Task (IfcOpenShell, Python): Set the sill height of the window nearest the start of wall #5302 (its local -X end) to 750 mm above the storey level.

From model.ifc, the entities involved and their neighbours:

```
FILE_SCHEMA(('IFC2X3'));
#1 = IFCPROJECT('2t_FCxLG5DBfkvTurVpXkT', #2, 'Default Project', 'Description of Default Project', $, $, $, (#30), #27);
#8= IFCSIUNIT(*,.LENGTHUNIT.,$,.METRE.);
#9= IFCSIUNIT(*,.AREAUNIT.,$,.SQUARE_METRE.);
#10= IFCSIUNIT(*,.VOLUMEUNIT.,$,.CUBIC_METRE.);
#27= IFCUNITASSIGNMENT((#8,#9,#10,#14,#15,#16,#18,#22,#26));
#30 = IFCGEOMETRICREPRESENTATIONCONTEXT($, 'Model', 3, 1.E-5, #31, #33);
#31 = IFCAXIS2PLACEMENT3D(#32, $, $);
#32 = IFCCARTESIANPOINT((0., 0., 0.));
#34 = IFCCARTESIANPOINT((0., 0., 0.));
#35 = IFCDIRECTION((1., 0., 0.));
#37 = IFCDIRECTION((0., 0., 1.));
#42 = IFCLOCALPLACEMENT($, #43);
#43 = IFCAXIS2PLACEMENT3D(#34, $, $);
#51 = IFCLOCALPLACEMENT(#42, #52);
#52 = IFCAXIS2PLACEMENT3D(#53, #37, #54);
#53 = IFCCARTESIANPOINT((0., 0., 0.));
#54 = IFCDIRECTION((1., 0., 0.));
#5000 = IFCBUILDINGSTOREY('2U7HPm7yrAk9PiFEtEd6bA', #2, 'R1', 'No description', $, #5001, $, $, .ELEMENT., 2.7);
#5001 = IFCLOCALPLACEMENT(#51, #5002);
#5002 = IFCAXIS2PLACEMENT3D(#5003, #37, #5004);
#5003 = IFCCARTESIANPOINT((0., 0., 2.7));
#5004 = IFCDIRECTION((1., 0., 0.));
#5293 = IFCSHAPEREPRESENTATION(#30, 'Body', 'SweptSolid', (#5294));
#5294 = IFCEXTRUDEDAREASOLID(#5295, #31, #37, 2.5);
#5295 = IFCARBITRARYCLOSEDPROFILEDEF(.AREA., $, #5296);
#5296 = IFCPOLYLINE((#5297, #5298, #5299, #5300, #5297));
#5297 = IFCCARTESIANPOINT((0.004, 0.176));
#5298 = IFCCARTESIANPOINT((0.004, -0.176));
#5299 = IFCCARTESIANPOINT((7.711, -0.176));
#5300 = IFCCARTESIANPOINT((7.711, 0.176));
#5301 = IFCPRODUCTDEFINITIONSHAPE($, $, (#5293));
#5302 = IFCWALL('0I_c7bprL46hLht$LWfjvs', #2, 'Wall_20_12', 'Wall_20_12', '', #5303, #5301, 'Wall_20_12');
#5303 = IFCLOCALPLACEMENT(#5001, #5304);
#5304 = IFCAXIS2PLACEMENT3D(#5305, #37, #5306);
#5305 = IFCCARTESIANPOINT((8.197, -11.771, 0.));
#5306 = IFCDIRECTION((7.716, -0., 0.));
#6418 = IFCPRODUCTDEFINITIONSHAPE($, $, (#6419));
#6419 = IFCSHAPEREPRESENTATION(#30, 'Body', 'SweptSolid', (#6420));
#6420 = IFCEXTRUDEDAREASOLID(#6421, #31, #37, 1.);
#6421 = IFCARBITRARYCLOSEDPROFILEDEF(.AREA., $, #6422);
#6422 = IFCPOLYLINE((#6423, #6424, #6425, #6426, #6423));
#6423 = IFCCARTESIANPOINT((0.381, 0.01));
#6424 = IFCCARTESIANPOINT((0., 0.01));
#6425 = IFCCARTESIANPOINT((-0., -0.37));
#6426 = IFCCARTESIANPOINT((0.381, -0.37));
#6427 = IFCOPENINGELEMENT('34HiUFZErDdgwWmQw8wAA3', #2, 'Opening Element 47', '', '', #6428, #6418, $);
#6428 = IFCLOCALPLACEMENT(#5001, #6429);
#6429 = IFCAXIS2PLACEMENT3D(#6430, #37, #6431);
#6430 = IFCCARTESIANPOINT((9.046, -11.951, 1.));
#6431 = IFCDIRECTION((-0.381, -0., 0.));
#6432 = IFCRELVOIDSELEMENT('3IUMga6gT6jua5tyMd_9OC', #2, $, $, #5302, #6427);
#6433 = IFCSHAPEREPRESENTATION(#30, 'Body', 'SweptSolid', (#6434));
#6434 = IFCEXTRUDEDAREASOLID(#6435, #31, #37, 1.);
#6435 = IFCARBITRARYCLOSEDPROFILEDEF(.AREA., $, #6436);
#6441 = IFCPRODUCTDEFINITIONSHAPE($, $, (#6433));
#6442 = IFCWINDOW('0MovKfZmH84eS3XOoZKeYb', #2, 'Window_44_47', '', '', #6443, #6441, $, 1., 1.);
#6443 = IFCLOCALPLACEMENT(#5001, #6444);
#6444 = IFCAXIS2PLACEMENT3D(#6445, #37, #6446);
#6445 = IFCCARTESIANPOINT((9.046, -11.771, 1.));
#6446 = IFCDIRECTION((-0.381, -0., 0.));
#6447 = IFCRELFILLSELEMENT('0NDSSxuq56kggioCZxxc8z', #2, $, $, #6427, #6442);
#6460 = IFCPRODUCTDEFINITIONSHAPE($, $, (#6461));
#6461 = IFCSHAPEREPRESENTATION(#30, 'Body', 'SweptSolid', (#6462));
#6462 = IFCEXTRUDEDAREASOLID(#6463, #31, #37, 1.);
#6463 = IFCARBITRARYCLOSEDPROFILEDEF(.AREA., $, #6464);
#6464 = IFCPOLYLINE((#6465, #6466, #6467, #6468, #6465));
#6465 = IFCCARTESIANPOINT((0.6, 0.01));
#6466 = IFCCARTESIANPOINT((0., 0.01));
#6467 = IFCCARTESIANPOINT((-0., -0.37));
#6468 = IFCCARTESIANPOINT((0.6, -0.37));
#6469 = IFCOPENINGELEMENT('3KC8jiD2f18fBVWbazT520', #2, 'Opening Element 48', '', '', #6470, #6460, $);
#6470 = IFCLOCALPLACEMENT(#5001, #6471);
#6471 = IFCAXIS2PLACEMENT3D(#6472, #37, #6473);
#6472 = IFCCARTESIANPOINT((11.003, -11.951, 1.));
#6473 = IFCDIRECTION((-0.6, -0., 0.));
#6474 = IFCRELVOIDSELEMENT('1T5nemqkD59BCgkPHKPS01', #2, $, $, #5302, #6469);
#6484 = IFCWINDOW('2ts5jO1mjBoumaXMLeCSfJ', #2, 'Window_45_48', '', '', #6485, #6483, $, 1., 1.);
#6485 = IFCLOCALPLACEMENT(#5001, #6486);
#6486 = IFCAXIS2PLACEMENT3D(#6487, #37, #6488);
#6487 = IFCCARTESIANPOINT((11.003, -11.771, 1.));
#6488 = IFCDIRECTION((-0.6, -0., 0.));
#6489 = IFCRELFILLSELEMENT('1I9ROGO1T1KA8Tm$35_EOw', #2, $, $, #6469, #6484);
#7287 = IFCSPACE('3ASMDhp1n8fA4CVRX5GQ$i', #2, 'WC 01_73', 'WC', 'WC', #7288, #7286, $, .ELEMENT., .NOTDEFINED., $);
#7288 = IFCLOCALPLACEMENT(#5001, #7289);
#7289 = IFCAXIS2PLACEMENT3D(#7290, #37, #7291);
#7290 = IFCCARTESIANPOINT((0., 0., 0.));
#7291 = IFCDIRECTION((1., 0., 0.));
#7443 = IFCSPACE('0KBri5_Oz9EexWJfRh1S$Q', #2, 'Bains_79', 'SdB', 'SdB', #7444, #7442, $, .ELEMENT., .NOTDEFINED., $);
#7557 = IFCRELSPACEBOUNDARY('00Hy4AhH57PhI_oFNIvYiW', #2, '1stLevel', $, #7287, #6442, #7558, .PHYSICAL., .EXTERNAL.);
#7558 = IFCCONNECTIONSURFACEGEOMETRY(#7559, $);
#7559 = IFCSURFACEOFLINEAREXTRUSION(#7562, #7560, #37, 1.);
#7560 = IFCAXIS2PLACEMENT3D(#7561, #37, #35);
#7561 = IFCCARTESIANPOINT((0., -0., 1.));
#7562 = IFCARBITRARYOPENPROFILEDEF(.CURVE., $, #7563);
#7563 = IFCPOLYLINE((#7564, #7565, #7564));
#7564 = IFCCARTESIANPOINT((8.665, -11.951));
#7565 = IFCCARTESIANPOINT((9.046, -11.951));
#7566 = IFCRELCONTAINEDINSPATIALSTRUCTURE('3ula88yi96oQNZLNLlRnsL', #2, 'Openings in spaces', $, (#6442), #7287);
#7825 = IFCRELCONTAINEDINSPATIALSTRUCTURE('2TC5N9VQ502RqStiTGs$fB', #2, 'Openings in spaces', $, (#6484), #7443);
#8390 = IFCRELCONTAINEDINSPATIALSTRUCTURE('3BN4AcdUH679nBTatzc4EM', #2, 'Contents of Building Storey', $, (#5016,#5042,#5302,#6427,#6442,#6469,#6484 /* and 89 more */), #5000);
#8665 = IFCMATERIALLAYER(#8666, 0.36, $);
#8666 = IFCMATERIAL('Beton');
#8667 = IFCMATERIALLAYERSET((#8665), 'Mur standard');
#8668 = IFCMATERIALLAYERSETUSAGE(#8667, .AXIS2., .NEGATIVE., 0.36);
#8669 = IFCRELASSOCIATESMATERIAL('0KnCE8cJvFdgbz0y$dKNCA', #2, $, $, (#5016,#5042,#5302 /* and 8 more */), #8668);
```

```python
import numpy as np
import ifcopenshell
import ifcopenshell.api.geometry
import ifcopenshell.geom
import ifcopenshell.util.element
import ifcopenshell.util.placement
import ifcopenshell.util.shape
import ifcopenshell.util.unit

model = ifcopenshell.open("model.ifc")
unit_scale = ifcopenshell.util.unit.calculate_unit_scale(model)

window = model.by_guid("0MovKfZmH84eS3XOoZKeYb")
opening = window.FillsVoids[0].RelatingOpeningElement
storey = ifcopenshell.util.element.get_container(window, ifc_class="IfcBuildingStorey")
level = ifcopenshell.util.placement.get_local_placement(storey.ObjectPlacement)[2, 3]

# The opening's origin need not be at the sill, so measure its lowest point.
shape = ifcopenshell.geom.create_shape(ifcopenshell.geom.settings(), opening)
bottom = ifcopenshell.util.shape.get_shape_bottom_elevation(shape, shape.geometry) / unit_scale
dz = level + 0.75 / unit_scale - bottom

shift = np.array([0.0, 0.0, dz])
# The window is not placed relative to its opening, so move both.
for product in (opening, window):
    matrix = ifcopenshell.util.placement.get_local_placement(product.ObjectPlacement)
    matrix[:3, 3] += shift
    ifcopenshell.api.geometry.edit_object_placement(model, product=product, matrix=matrix, is_si=False)

# Space boundary surfaces are stored in each space's coordinates; move them too.
for rel in window.ProvidesBoundaries:
    if not rel.ConnectionGeometry:
        continue
    surface = rel.ConnectionGeometry.SurfaceOnRelatingElement
    space_matrix = ifcopenshell.util.placement.get_local_placement(rel.RelatingSpace.ObjectPlacement)
    point = np.array(surface.Position.Location.Coordinates) + space_matrix[:3, :3].T @ shift
    surface.Position = model.createIfcAxis2Placement3D(
        model.createIfcCartesianPoint(point.tolist()), surface.Position.Axis, surface.Position.RefDirection
    )

print(f"moved by {dz * unit_scale:+.3f} m")

model.write("model_rev.ifc")
```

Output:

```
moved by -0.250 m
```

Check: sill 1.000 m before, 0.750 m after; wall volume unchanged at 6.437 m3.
